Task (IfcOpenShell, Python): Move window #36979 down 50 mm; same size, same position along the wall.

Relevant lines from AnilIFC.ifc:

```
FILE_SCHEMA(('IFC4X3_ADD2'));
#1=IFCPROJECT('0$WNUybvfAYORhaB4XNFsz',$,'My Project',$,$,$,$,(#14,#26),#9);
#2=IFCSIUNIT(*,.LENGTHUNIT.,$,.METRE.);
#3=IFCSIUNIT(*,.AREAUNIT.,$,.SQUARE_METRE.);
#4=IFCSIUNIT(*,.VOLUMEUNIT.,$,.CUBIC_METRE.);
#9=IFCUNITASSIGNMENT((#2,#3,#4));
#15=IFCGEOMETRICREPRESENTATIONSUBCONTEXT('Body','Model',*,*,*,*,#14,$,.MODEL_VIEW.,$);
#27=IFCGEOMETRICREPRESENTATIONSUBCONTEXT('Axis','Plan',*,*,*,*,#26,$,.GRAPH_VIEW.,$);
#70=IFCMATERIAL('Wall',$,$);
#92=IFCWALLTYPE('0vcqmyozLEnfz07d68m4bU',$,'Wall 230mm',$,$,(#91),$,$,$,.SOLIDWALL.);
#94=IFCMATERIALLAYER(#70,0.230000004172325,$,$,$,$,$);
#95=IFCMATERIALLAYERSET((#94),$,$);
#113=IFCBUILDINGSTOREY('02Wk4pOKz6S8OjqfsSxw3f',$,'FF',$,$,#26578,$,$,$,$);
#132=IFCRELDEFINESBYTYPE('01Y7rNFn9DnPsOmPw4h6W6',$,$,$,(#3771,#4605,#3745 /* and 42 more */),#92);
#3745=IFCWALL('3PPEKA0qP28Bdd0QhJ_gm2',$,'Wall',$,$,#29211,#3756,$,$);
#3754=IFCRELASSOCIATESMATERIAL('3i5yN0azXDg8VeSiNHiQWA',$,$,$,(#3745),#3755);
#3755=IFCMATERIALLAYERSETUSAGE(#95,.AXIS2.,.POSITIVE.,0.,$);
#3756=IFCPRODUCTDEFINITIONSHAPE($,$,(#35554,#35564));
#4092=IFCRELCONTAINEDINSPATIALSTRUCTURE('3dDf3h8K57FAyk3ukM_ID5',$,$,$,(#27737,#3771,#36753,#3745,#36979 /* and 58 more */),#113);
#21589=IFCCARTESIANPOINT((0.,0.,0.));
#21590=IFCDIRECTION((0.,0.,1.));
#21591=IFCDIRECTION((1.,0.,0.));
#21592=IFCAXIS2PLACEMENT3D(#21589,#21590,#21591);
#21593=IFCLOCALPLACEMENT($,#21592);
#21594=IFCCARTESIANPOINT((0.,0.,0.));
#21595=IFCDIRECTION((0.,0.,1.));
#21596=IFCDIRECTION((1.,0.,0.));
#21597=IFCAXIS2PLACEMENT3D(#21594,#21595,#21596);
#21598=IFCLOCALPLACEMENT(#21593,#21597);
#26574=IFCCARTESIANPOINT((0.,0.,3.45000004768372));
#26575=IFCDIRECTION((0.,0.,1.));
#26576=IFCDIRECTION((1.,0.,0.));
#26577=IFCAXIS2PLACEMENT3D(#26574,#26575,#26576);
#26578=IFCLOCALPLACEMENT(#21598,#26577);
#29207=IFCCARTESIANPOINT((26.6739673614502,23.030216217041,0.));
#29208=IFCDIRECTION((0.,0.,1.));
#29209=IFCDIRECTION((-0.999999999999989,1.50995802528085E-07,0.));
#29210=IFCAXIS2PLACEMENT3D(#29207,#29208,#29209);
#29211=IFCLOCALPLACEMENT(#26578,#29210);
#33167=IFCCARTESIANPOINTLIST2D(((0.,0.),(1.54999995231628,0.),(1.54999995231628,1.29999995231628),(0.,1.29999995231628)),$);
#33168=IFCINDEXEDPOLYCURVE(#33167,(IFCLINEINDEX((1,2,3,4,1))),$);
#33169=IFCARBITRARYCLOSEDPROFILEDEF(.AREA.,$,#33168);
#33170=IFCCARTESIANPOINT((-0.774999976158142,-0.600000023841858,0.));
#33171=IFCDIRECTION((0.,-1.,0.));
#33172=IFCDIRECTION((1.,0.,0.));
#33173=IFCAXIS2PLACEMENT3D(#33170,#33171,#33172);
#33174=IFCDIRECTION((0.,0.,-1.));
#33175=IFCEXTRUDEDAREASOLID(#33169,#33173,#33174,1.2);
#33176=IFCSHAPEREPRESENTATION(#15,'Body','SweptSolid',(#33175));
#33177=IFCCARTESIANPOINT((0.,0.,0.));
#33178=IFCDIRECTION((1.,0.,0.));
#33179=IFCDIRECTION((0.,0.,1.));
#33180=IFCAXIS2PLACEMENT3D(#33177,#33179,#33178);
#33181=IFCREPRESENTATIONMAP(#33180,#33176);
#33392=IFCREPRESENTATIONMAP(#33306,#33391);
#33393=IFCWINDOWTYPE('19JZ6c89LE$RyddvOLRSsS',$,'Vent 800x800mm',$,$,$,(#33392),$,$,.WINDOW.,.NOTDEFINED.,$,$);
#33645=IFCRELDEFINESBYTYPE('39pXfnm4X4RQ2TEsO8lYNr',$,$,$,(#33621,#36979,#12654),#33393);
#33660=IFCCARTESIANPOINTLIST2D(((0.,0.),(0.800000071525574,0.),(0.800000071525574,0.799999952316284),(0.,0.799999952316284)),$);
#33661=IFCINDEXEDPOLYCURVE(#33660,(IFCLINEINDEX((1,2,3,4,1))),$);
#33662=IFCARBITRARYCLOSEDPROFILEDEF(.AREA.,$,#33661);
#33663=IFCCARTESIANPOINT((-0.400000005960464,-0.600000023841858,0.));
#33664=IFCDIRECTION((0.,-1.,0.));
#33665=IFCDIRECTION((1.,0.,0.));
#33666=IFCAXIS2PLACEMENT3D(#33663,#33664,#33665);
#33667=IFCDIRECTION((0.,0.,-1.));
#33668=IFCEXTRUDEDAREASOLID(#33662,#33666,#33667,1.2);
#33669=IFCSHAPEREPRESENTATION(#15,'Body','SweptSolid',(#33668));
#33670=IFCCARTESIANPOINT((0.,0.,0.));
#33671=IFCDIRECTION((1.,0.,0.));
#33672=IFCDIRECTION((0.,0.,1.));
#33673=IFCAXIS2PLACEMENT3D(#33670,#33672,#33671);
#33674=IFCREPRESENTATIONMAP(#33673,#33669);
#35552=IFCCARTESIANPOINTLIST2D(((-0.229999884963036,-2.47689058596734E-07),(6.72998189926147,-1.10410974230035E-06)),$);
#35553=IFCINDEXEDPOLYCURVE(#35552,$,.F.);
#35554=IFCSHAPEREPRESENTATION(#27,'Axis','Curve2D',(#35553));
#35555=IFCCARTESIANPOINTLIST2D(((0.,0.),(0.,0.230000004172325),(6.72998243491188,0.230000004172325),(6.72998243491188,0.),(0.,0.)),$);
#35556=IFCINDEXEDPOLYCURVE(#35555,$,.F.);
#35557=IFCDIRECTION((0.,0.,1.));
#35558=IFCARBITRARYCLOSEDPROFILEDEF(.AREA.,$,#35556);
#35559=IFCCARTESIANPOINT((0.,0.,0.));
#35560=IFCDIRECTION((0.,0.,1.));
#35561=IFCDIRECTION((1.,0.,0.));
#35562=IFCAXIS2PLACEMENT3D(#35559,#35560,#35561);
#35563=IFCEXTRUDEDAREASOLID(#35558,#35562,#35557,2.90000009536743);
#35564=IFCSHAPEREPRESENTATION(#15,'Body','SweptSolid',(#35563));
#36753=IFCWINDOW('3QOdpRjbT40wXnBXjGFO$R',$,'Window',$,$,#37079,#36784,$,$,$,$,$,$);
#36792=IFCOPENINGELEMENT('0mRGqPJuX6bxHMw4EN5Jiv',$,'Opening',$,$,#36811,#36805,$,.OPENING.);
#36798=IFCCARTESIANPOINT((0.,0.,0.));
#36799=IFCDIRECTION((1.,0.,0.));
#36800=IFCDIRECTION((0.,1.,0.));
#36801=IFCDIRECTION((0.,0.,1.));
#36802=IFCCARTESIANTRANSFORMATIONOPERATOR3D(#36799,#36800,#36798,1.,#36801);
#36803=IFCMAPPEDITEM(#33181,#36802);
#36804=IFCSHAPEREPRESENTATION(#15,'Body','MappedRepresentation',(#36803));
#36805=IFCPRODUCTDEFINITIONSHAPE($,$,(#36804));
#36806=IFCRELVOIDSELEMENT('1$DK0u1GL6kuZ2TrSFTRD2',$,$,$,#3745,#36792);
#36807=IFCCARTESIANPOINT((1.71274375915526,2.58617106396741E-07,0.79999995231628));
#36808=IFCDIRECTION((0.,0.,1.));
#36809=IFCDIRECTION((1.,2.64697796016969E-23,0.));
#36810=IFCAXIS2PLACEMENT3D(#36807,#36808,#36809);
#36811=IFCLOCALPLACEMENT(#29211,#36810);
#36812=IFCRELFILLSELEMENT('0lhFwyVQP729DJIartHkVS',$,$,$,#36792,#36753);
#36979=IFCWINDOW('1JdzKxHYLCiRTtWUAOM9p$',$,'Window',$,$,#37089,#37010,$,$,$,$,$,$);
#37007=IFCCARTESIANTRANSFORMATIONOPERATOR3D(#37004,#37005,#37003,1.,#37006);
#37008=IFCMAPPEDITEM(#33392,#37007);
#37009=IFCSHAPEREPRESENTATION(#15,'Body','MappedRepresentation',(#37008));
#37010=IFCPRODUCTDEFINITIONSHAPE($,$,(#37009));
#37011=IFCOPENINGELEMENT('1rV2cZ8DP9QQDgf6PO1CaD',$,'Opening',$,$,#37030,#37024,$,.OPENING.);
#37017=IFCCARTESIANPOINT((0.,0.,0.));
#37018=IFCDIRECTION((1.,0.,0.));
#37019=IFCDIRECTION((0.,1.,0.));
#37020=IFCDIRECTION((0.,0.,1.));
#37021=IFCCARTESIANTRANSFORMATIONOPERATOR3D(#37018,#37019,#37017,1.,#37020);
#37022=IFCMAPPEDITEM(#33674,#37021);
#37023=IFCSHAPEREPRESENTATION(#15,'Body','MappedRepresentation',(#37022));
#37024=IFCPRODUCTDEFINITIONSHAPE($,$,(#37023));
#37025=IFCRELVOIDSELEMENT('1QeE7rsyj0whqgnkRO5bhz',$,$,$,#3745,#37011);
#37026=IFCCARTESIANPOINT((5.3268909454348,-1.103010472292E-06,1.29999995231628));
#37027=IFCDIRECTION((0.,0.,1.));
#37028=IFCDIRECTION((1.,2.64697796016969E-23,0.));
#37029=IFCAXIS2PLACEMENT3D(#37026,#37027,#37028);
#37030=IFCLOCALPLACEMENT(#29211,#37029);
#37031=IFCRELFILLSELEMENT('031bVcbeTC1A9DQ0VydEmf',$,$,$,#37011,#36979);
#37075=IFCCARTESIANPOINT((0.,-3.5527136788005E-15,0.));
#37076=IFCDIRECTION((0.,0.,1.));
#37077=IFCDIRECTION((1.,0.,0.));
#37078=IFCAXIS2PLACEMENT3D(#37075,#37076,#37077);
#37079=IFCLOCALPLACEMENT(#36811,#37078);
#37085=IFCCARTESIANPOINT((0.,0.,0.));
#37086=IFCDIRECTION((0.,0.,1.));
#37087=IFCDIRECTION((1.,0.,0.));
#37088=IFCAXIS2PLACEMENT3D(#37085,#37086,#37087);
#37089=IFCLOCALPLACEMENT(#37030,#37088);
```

```python
import numpy as np
import ifcopenshell
import ifcopenshell.api.geometry
import ifcopenshell.util.placement
import ifcopenshell.util.unit

model = ifcopenshell.open("AnilIFC.ifc")
unit_scale = ifcopenshell.util.unit.calculate_unit_scale(model)

window = model.by_guid("1JdzKxHYLCiRTtWUAOM9p$")
opening = window.FillsVoids[0].RelatingOpeningElement
dz = -0.05 / unit_scale

shift = np.array([0.0, 0.0, dz])
# The window is placed relative to its opening, so it follows when the opening moves.
matrix = ifcopenshell.util.placement.get_local_placement(opening.ObjectPlacement)
matrix[:3, 3] += shift
ifcopenshell.api.geometry.edit_object_placement(
    model, product=opening, matrix=matrix, is_si=False, should_transform_children=True
)

print(f"moved by {dz * unit_scale:+.3f} m")

model.write("AnilIFC_rev.ifc")
```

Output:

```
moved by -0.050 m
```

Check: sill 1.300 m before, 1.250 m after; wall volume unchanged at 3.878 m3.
